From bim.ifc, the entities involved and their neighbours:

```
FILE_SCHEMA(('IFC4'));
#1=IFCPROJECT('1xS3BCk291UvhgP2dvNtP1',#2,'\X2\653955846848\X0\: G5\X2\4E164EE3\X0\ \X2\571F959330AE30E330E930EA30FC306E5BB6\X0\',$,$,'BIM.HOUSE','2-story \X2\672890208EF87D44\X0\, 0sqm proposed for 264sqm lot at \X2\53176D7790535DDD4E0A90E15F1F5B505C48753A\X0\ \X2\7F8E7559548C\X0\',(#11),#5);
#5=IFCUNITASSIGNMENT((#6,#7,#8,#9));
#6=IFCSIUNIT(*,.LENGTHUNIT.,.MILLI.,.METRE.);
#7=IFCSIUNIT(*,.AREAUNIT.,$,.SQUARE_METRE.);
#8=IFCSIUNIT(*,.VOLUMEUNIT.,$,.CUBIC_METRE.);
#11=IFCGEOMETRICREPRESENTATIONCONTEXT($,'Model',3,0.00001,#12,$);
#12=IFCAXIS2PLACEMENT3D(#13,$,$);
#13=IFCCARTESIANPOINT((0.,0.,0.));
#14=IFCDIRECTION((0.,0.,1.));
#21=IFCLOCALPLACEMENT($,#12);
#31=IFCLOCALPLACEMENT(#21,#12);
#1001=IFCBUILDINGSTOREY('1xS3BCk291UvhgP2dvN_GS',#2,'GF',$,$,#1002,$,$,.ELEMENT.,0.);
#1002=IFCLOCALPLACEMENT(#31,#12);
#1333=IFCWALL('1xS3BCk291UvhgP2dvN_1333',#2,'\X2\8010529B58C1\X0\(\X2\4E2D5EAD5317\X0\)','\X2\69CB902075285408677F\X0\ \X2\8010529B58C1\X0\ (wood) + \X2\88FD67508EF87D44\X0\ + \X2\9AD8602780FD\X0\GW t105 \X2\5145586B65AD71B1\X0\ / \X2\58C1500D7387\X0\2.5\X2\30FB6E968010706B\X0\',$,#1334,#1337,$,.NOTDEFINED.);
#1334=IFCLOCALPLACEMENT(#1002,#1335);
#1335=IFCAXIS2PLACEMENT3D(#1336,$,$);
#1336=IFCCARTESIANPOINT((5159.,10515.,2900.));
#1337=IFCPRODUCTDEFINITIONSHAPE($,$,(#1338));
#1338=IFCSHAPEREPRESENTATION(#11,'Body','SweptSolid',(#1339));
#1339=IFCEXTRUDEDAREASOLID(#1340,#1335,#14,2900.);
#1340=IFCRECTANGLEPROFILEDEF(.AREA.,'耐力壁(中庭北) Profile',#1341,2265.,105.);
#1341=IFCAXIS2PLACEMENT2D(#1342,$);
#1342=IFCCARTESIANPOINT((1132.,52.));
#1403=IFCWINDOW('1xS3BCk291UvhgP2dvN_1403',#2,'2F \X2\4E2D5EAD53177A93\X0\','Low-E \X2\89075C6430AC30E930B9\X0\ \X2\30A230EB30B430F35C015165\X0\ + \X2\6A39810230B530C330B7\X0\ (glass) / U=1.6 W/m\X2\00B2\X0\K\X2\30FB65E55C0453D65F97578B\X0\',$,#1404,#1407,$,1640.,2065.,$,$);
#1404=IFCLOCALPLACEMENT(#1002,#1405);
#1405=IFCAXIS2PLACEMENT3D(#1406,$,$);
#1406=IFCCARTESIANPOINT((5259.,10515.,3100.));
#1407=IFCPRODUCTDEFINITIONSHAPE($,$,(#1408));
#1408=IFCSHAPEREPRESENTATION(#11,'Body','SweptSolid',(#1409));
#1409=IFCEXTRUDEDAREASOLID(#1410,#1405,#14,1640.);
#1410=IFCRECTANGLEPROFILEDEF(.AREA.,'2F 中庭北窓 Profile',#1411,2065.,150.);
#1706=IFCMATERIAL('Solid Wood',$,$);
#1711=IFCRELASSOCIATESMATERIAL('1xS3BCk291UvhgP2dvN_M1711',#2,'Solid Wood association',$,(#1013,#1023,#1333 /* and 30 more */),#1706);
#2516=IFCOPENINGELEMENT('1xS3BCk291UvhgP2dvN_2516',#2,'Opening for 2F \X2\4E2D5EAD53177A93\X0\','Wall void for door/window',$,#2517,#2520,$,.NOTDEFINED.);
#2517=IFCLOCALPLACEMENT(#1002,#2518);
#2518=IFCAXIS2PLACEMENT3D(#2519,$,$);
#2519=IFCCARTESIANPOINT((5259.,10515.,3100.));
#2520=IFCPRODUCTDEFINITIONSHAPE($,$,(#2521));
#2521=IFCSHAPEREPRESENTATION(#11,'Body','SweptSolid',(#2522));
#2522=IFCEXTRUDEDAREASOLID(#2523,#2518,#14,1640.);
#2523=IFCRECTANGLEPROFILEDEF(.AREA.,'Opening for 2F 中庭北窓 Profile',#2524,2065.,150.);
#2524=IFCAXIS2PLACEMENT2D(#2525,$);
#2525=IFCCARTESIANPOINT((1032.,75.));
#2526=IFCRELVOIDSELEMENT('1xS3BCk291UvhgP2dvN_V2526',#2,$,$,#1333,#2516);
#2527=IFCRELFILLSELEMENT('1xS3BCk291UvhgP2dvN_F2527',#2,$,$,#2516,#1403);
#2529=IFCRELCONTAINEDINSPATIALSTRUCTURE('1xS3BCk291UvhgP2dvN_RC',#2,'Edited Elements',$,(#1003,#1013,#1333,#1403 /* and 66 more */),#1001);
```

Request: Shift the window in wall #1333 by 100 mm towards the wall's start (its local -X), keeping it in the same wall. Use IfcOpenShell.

```python
import ifcopenshell
import ifcopenshell.api.geometry
import ifcopenshell.util.placement
import ifcopenshell.util.unit

model = ifcopenshell.open("bim.ifc")
unit_scale = ifcopenshell.util.unit.calculate_unit_scale(model)

window = model.by_guid("1xS3BCk291UvhgP2dvN_1403")
opening = window.FillsVoids[0].RelatingOpeningElement
wall = opening.VoidsElements[0].RelatingBuildingElement

wall_matrix = ifcopenshell.util.placement.get_local_placement(wall.ObjectPlacement)
shift = wall_matrix[:3, 0] * -0.1 / unit_scale
before = ifcopenshell.util.placement.get_local_placement(window.ObjectPlacement)[:3, 3].copy()

# The window is not placed relative to its opening, so move both.
for product in (opening, window):
    matrix = ifcopenshell.util.placement.get_local_placement(product.ObjectPlacement)
    matrix[:3, 3] += shift
    ifcopenshell.api.geometry.edit_object_placement(model, product=product, matrix=matrix, is_si=False)

after = ifcopenshell.util.placement.get_local_placement(window.ObjectPlacement)[:3, 3]
print("window moved by", (after - before).round(3) + 0.0)

model.write("bim_v2.ifc")
```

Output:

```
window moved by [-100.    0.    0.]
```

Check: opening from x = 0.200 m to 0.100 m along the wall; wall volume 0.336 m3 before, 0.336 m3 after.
